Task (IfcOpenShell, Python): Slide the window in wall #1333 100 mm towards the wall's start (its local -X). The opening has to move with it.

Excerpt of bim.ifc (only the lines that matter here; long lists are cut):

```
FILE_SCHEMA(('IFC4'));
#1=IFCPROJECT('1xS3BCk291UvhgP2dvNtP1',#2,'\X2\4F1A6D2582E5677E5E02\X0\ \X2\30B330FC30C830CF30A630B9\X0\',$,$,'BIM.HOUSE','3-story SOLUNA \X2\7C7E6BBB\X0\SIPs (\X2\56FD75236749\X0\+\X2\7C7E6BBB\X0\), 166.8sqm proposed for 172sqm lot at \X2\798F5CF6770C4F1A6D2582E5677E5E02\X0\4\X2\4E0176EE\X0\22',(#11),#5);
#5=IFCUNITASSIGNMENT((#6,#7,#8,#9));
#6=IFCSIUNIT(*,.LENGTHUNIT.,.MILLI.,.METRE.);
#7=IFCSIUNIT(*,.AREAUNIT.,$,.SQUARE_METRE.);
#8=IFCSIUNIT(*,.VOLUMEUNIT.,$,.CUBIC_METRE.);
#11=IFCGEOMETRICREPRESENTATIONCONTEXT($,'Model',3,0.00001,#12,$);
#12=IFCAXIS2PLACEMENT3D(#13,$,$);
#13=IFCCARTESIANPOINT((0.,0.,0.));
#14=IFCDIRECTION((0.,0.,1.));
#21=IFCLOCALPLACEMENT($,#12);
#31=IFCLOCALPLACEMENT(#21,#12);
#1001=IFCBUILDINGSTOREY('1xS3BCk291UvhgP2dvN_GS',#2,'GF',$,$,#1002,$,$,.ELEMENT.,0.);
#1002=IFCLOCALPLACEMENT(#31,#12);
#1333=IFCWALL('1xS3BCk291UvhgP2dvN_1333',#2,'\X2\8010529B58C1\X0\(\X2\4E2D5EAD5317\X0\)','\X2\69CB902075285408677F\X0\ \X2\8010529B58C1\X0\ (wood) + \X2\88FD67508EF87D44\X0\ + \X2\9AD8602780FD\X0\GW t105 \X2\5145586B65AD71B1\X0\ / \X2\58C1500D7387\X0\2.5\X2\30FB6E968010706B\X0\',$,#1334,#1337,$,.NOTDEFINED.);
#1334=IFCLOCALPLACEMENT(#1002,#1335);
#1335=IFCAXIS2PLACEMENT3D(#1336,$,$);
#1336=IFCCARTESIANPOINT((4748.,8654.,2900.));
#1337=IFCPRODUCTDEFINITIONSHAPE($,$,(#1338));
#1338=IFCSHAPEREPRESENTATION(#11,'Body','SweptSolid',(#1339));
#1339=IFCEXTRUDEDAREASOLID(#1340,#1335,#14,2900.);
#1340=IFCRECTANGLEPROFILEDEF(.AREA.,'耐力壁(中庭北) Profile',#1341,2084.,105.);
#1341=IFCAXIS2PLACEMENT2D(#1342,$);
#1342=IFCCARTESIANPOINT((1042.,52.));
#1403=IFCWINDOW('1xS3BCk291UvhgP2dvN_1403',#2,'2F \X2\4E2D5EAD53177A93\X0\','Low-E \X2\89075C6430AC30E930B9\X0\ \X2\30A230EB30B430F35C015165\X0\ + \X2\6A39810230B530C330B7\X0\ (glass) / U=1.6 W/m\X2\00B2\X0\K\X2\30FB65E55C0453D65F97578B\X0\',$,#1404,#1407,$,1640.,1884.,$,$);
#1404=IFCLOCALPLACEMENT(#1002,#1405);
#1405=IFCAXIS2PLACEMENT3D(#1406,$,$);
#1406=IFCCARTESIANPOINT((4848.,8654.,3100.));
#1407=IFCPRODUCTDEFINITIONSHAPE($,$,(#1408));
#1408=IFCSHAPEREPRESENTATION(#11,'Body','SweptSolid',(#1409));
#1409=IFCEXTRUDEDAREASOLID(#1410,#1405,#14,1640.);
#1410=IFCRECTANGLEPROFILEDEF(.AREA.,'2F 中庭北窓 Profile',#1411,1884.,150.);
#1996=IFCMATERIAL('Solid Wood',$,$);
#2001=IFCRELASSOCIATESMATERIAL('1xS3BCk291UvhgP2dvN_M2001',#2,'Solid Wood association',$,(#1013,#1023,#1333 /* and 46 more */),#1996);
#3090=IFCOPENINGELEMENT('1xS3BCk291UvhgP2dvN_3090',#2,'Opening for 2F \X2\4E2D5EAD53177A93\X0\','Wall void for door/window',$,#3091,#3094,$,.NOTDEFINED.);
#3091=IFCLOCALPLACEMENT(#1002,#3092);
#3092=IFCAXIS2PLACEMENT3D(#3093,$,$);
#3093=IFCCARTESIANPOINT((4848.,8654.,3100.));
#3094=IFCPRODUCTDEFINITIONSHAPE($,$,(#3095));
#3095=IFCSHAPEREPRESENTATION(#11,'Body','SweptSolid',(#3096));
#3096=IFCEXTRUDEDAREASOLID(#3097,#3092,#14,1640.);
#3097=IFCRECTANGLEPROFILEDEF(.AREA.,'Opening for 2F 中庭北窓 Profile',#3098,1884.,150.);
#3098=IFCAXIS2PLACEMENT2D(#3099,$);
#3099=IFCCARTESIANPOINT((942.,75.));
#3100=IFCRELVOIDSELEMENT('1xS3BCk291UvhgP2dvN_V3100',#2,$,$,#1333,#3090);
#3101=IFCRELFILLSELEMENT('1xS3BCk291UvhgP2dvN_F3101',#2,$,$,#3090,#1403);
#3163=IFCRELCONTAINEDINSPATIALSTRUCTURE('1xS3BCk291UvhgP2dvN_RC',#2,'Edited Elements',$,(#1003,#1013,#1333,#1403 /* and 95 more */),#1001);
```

```python
import ifcopenshell
import ifcopenshell.api.geometry
import ifcopenshell.util.placement

model = ifcopenshell.open("bim.ifc")

window = model.by_guid("1xS3BCk291UvhgP2dvN_1403")
opening = window.FillsVoids[0].RelatingOpeningElement
wall = opening.VoidsElements[0].RelatingBuildingElement

wall_matrix = ifcopenshell.util.placement.get_local_placement(wall.ObjectPlacement)
shift = wall_matrix[:3, 0] * -100.0
before = ifcopenshell.util.placement.get_local_placement(window.ObjectPlacement)[:3, 3].copy()

# The window is not placed relative to its opening, so move both.
for product in (opening, window):
    matrix = ifcopenshell.util.placement.get_local_placement(product.ObjectPlacement)
    matrix[:3, 3] += shift
    ifcopenshell.api.geometry.edit_object_placement(model, product=product, matrix=matrix, is_si=False)

after = ifcopenshell.util.placement.get_local_placement(window.ObjectPlacement)[:3, 3]
print("window moved by", (after - before).round(3) + 0.0)

model.write("bim_v2.ifc")
```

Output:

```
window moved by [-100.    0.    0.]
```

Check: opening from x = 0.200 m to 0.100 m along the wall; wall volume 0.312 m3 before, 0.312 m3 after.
